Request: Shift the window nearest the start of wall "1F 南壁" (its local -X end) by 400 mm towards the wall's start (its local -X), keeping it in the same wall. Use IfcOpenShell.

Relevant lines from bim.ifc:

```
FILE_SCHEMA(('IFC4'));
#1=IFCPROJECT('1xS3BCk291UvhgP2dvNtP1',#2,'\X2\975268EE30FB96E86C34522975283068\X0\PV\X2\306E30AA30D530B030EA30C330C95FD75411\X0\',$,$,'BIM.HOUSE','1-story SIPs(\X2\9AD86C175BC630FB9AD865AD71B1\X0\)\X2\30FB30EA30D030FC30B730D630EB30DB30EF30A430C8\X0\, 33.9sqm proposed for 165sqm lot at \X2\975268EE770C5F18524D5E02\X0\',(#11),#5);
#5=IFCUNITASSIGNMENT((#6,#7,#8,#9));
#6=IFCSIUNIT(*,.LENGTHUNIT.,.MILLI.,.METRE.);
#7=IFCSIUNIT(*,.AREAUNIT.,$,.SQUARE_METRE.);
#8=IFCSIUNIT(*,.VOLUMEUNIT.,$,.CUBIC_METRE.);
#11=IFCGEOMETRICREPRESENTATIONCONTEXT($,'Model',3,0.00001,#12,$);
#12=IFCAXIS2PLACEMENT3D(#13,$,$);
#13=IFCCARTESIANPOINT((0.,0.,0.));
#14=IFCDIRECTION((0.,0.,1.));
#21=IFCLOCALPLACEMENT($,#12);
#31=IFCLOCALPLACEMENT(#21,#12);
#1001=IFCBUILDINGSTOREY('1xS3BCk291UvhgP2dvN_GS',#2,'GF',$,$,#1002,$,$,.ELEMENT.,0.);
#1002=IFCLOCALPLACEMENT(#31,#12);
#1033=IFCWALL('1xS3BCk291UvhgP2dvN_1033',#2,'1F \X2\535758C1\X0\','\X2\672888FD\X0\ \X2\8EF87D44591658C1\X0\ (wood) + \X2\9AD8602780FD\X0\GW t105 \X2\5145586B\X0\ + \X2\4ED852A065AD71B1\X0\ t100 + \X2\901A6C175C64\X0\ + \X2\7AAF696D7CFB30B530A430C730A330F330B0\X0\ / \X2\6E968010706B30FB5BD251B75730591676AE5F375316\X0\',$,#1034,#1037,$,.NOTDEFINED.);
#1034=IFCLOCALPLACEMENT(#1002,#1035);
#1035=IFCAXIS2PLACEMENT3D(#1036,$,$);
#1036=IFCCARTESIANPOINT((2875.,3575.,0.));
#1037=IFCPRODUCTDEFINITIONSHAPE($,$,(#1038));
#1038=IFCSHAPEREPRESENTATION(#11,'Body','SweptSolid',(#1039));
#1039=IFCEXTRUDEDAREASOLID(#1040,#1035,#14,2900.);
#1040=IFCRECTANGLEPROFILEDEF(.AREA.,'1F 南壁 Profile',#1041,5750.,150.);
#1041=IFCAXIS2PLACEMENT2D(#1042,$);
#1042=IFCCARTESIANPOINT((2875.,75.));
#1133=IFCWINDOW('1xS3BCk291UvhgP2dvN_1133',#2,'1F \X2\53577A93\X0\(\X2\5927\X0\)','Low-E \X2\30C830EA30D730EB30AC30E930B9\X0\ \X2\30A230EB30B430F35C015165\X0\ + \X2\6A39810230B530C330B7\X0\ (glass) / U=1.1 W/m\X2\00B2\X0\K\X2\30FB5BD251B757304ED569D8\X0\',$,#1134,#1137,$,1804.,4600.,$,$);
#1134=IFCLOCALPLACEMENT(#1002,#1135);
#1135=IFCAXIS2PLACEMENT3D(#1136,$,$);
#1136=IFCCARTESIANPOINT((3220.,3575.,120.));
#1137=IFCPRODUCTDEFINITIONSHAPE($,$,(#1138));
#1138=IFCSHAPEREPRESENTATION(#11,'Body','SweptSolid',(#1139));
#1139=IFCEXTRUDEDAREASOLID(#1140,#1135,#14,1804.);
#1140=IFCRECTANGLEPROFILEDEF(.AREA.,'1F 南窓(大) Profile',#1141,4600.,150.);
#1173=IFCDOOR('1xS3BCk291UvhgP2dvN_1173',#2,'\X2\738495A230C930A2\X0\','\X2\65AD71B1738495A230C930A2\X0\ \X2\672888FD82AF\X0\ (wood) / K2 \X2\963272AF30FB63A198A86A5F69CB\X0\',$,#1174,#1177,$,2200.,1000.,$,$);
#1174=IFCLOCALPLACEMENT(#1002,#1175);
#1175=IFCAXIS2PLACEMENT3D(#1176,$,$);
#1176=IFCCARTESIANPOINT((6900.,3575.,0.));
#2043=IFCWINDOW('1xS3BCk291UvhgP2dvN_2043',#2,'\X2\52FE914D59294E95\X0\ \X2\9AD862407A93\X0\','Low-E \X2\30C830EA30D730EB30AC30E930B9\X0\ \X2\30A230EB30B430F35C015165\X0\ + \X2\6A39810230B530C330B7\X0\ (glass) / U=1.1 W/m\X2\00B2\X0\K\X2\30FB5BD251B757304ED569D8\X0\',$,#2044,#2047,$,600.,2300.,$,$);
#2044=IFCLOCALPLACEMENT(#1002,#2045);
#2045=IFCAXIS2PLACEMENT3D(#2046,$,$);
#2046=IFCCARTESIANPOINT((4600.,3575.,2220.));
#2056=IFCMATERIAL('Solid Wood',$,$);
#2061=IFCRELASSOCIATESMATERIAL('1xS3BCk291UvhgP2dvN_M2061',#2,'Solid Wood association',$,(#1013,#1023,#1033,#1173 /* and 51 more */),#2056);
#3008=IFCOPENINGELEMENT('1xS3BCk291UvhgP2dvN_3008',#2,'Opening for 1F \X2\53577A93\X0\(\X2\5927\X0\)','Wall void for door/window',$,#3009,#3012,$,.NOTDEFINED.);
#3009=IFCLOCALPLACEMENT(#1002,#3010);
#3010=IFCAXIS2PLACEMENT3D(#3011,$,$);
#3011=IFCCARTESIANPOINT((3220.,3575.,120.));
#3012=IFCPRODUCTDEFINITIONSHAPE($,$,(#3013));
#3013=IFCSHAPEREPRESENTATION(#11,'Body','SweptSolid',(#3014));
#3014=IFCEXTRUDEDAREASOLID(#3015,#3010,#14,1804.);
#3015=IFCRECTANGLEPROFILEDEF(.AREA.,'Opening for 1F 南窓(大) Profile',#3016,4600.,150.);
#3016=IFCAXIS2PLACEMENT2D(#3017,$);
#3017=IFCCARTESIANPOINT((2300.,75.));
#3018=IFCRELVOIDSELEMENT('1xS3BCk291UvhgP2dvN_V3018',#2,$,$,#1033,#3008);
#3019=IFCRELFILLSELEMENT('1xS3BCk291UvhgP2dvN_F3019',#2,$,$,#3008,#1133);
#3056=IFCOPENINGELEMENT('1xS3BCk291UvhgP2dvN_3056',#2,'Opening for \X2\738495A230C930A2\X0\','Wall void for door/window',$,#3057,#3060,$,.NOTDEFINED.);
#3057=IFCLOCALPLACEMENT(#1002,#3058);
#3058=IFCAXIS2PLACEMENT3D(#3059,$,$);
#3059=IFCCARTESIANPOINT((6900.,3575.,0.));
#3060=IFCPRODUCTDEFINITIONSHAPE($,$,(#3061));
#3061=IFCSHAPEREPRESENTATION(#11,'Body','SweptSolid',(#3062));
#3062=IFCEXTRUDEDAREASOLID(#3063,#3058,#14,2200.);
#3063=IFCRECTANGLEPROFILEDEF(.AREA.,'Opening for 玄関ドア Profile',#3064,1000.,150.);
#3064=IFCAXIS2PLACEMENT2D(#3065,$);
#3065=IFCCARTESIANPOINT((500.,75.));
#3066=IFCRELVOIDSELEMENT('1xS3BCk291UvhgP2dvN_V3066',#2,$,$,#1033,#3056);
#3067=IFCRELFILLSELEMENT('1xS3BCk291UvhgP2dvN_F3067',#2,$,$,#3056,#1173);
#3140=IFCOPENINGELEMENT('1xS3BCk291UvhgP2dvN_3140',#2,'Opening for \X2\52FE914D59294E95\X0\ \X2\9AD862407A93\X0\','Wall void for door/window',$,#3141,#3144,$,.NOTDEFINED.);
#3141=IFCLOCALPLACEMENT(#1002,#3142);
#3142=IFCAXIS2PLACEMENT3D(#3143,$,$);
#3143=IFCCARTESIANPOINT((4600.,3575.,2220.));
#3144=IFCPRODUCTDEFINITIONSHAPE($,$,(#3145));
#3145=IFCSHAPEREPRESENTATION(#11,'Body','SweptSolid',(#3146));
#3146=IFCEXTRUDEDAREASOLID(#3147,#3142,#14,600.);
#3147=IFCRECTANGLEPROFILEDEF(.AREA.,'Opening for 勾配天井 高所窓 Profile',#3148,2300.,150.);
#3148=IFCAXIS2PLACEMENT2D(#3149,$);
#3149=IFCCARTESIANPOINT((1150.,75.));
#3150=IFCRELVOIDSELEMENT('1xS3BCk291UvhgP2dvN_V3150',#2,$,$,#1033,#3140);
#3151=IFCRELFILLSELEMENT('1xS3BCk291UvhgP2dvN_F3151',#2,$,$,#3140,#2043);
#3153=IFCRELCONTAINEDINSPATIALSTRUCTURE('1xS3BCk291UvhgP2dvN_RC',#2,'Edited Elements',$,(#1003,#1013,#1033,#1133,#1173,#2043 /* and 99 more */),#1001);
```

```python
import ifcopenshell
import ifcopenshell.api.geometry
import ifcopenshell.util.placement
import ifcopenshell.util.unit

model = ifcopenshell.open("bim.ifc")
unit_scale = ifcopenshell.util.unit.calculate_unit_scale(model)

window = model.by_guid("1xS3BCk291UvhgP2dvN_1133")
opening = window.FillsVoids[0].RelatingOpeningElement
wall = opening.VoidsElements[0].RelatingBuildingElement

wall_matrix = ifcopenshell.util.placement.get_local_placement(wall.ObjectPlacement)
shift = wall_matrix[:3, 0] * -0.4 / unit_scale
before = ifcopenshell.util.placement.get_local_placement(window.ObjectPlacement)[:3, 3].copy()

# The window is not placed relative to its opening, so move both.
for product in (opening, window):
    matrix = ifcopenshell.util.placement.get_local_placement(product.ObjectPlacement)
    matrix[:3, 3] += shift
    ifcopenshell.api.geometry.edit_object_placement(model, product=product, matrix=matrix, is_si=False)

after = ifcopenshell.util.placement.get_local_placement(window.ObjectPlacement)[:3, 3]
print("window moved by", (after - before).round(3) + 0.0)

model.write("bim_edited.ifc")
```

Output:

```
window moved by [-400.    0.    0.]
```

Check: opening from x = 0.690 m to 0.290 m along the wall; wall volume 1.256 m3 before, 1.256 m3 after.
